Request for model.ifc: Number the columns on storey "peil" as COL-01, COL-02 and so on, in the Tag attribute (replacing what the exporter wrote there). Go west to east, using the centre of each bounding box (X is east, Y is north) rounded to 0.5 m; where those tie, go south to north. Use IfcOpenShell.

First a look at what the model holds.

```python
import ifcopenshell
import ifcopenshell.util.element
import ifcopenshell.util.placement

model = ifcopenshell.open("model.ifc")
print(model.schema)
storey = next(s for s in model.by_type("IfcBuildingStorey") if s.Name == "peil")
columns = [e for e in ifcopenshell.util.element.get_decomposition(storey) if e.is_a("IfcColumn")]
for e in sorted(columns, key=lambda e: e.id()):
    origin = ifcopenshell.util.placement.get_local_placement(e.ObjectPlacement)[:3, 3]
    print(e.id(), e.Tag, e.Name, origin.round(2) + 0.0, sep=" | ")
```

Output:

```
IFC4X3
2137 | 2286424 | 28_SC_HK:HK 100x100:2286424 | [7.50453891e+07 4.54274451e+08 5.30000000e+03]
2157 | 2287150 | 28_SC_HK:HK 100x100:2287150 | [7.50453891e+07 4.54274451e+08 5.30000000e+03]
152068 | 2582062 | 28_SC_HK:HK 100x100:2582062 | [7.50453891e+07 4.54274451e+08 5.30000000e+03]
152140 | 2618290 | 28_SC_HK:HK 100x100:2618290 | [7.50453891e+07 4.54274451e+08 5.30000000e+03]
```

```python
import ifcopenshell
import ifcopenshell.geom
import ifcopenshell.util.element
import ifcopenshell.util.shape

model = ifcopenshell.open("model.ifc")
settings = ifcopenshell.geom.settings()
settings.set("use-world-coords", True)


def centre(element):
    shape = ifcopenshell.geom.create_shape(settings, element)
    return ifcopenshell.util.shape.get_bbox_centroid(shape.geometry)


storey = next(s for s in model.by_type("IfcBuildingStorey") if s.Name == "peil")
columns = [e for e in ifcopenshell.util.element.get_decomposition(storey) if e.is_a("IfcColumn")]

# Insertion points can sit at a corner or the storey origin, so sort by the geometry (in metres).
centres = {e: centre(e) for e in columns}
columns.sort(key=lambda e: (round(centres[e][0] / 0.5), centres[e][1]))

for i, e in enumerate(columns, start=1):
    number = f"COL-{i:02d}"
    e.Tag = number
    print(e.id(), number)

model.write("model_rev.ifc")
```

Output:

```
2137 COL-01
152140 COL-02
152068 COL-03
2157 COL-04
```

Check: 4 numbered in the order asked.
